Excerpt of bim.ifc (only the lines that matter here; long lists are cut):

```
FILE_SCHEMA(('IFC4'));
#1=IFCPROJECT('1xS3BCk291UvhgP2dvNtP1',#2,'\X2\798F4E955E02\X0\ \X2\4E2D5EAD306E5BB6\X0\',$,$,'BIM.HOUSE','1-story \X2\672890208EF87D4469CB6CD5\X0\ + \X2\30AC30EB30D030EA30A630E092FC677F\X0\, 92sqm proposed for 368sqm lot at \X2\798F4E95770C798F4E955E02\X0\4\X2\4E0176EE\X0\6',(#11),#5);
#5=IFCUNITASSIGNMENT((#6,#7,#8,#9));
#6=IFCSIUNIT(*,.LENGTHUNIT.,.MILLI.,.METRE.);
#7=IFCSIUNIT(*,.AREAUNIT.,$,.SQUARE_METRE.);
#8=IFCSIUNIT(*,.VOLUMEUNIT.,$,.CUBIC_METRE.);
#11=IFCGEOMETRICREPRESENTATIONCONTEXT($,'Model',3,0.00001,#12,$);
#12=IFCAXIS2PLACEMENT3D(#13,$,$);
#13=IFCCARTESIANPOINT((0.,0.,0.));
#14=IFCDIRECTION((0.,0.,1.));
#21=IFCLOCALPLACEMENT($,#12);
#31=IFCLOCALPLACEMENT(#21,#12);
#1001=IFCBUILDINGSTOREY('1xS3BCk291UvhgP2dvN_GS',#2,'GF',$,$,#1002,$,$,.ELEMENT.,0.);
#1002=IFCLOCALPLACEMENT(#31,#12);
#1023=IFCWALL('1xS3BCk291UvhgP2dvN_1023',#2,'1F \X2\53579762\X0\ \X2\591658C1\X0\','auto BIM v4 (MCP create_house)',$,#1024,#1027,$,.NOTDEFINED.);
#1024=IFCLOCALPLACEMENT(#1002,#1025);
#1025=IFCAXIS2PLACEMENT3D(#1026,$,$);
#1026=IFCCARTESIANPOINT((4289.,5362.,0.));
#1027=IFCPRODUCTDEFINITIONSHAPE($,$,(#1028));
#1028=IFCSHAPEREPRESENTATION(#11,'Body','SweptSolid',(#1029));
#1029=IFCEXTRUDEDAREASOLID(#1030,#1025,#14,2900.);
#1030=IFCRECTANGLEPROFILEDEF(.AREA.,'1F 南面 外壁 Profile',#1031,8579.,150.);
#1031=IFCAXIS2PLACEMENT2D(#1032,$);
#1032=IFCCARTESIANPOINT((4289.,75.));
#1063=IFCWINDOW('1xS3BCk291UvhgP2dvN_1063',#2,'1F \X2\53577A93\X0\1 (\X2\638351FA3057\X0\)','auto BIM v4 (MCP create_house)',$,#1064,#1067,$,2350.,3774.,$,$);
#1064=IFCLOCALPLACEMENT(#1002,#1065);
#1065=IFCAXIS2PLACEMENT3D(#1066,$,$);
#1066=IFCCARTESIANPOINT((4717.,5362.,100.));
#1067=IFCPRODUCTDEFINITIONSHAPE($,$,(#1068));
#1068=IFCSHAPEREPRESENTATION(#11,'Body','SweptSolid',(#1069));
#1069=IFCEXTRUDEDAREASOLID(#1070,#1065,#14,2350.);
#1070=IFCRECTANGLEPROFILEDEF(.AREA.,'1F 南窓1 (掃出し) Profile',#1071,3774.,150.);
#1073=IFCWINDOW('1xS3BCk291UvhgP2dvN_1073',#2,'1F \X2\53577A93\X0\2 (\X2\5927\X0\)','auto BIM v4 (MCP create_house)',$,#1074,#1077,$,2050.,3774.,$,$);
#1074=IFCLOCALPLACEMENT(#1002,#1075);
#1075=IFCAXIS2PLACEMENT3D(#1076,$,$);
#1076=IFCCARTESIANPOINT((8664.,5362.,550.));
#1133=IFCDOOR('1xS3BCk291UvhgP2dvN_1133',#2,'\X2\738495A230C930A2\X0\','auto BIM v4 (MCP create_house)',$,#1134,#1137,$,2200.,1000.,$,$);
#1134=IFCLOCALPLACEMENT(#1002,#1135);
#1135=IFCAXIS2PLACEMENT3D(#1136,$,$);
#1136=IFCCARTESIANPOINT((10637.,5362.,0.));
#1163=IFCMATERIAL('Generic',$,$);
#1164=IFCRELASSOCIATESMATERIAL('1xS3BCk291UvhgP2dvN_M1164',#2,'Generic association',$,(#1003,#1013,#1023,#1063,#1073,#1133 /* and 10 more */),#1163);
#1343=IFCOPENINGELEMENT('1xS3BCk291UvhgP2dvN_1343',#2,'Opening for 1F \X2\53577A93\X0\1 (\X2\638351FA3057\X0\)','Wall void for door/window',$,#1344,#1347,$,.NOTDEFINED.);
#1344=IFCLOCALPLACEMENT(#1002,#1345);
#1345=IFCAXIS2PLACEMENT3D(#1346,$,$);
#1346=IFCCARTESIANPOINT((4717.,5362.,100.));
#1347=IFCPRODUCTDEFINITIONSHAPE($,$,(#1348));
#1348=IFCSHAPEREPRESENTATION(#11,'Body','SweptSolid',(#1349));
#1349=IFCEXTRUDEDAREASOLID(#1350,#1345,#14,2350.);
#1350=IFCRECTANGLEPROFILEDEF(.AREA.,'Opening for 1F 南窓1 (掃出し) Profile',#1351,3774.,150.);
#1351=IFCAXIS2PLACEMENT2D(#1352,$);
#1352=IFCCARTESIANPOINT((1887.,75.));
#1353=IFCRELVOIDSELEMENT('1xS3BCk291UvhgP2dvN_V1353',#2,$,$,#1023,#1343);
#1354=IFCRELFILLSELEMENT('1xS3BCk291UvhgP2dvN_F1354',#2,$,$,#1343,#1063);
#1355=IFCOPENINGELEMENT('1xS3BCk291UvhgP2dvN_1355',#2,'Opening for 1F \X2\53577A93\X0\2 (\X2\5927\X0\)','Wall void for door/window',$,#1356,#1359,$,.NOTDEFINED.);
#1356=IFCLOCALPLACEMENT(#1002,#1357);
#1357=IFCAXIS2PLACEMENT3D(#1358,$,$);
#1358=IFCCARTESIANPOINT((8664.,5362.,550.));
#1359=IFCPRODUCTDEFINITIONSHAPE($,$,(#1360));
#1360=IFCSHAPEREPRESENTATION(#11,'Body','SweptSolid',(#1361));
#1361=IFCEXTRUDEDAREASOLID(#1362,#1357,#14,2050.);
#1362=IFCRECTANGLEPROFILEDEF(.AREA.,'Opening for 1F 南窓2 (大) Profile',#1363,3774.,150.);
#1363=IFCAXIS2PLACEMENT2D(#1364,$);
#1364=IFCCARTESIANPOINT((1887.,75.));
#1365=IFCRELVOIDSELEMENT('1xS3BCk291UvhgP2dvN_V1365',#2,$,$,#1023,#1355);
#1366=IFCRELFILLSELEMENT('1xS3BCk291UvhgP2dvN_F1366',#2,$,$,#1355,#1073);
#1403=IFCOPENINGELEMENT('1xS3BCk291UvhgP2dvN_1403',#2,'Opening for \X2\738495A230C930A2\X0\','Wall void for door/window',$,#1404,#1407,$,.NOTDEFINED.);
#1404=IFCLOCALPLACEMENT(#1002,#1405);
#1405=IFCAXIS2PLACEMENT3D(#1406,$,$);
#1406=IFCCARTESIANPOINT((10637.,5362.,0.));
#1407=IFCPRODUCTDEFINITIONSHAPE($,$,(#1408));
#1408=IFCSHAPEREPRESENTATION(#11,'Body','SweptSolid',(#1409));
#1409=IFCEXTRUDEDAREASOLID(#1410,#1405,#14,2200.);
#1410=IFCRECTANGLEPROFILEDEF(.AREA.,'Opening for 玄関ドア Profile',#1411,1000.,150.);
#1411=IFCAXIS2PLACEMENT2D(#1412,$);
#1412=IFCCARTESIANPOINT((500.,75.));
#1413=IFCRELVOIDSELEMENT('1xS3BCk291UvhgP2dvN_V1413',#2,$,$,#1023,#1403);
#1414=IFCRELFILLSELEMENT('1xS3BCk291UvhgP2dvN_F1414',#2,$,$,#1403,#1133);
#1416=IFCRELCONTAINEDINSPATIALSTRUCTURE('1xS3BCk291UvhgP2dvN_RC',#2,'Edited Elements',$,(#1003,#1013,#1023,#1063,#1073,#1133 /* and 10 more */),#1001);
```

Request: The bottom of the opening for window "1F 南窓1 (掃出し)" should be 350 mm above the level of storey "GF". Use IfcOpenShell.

```python
import numpy as np
import ifcopenshell
import ifcopenshell.api.geometry
import ifcopenshell.geom
import ifcopenshell.util.element
import ifcopenshell.util.placement
import ifcopenshell.util.shape
import ifcopenshell.util.unit

model = ifcopenshell.open("bim.ifc")
unit_scale = ifcopenshell.util.unit.calculate_unit_scale(model)

window = model.by_guid("1xS3BCk291UvhgP2dvN_1063")
opening = window.FillsVoids[0].RelatingOpeningElement
storey = ifcopenshell.util.element.get_container(window, ifc_class="IfcBuildingStorey")
level = ifcopenshell.util.placement.get_local_placement(storey.ObjectPlacement)[2, 3]

# The opening's origin need not be at the sill, so measure its lowest point.
shape = ifcopenshell.geom.create_shape(ifcopenshell.geom.settings(), opening)
bottom = ifcopenshell.util.shape.get_shape_bottom_elevation(shape, shape.geometry) / unit_scale
dz = level + 0.35 / unit_scale - bottom

shift = np.array([0.0, 0.0, dz])
# The window is not placed relative to its opening, so move both.
for product in (opening, window):
    matrix = ifcopenshell.util.placement.get_local_placement(product.ObjectPlacement)
    matrix[:3, 3] += shift
    ifcopenshell.api.geometry.edit_object_placement(model, product=product, matrix=matrix, is_si=False)

print(f"moved by {dz * unit_scale:+.3f} m")

model.write("bim-out.ifc")
```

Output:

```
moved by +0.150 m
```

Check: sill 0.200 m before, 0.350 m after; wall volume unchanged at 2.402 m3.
